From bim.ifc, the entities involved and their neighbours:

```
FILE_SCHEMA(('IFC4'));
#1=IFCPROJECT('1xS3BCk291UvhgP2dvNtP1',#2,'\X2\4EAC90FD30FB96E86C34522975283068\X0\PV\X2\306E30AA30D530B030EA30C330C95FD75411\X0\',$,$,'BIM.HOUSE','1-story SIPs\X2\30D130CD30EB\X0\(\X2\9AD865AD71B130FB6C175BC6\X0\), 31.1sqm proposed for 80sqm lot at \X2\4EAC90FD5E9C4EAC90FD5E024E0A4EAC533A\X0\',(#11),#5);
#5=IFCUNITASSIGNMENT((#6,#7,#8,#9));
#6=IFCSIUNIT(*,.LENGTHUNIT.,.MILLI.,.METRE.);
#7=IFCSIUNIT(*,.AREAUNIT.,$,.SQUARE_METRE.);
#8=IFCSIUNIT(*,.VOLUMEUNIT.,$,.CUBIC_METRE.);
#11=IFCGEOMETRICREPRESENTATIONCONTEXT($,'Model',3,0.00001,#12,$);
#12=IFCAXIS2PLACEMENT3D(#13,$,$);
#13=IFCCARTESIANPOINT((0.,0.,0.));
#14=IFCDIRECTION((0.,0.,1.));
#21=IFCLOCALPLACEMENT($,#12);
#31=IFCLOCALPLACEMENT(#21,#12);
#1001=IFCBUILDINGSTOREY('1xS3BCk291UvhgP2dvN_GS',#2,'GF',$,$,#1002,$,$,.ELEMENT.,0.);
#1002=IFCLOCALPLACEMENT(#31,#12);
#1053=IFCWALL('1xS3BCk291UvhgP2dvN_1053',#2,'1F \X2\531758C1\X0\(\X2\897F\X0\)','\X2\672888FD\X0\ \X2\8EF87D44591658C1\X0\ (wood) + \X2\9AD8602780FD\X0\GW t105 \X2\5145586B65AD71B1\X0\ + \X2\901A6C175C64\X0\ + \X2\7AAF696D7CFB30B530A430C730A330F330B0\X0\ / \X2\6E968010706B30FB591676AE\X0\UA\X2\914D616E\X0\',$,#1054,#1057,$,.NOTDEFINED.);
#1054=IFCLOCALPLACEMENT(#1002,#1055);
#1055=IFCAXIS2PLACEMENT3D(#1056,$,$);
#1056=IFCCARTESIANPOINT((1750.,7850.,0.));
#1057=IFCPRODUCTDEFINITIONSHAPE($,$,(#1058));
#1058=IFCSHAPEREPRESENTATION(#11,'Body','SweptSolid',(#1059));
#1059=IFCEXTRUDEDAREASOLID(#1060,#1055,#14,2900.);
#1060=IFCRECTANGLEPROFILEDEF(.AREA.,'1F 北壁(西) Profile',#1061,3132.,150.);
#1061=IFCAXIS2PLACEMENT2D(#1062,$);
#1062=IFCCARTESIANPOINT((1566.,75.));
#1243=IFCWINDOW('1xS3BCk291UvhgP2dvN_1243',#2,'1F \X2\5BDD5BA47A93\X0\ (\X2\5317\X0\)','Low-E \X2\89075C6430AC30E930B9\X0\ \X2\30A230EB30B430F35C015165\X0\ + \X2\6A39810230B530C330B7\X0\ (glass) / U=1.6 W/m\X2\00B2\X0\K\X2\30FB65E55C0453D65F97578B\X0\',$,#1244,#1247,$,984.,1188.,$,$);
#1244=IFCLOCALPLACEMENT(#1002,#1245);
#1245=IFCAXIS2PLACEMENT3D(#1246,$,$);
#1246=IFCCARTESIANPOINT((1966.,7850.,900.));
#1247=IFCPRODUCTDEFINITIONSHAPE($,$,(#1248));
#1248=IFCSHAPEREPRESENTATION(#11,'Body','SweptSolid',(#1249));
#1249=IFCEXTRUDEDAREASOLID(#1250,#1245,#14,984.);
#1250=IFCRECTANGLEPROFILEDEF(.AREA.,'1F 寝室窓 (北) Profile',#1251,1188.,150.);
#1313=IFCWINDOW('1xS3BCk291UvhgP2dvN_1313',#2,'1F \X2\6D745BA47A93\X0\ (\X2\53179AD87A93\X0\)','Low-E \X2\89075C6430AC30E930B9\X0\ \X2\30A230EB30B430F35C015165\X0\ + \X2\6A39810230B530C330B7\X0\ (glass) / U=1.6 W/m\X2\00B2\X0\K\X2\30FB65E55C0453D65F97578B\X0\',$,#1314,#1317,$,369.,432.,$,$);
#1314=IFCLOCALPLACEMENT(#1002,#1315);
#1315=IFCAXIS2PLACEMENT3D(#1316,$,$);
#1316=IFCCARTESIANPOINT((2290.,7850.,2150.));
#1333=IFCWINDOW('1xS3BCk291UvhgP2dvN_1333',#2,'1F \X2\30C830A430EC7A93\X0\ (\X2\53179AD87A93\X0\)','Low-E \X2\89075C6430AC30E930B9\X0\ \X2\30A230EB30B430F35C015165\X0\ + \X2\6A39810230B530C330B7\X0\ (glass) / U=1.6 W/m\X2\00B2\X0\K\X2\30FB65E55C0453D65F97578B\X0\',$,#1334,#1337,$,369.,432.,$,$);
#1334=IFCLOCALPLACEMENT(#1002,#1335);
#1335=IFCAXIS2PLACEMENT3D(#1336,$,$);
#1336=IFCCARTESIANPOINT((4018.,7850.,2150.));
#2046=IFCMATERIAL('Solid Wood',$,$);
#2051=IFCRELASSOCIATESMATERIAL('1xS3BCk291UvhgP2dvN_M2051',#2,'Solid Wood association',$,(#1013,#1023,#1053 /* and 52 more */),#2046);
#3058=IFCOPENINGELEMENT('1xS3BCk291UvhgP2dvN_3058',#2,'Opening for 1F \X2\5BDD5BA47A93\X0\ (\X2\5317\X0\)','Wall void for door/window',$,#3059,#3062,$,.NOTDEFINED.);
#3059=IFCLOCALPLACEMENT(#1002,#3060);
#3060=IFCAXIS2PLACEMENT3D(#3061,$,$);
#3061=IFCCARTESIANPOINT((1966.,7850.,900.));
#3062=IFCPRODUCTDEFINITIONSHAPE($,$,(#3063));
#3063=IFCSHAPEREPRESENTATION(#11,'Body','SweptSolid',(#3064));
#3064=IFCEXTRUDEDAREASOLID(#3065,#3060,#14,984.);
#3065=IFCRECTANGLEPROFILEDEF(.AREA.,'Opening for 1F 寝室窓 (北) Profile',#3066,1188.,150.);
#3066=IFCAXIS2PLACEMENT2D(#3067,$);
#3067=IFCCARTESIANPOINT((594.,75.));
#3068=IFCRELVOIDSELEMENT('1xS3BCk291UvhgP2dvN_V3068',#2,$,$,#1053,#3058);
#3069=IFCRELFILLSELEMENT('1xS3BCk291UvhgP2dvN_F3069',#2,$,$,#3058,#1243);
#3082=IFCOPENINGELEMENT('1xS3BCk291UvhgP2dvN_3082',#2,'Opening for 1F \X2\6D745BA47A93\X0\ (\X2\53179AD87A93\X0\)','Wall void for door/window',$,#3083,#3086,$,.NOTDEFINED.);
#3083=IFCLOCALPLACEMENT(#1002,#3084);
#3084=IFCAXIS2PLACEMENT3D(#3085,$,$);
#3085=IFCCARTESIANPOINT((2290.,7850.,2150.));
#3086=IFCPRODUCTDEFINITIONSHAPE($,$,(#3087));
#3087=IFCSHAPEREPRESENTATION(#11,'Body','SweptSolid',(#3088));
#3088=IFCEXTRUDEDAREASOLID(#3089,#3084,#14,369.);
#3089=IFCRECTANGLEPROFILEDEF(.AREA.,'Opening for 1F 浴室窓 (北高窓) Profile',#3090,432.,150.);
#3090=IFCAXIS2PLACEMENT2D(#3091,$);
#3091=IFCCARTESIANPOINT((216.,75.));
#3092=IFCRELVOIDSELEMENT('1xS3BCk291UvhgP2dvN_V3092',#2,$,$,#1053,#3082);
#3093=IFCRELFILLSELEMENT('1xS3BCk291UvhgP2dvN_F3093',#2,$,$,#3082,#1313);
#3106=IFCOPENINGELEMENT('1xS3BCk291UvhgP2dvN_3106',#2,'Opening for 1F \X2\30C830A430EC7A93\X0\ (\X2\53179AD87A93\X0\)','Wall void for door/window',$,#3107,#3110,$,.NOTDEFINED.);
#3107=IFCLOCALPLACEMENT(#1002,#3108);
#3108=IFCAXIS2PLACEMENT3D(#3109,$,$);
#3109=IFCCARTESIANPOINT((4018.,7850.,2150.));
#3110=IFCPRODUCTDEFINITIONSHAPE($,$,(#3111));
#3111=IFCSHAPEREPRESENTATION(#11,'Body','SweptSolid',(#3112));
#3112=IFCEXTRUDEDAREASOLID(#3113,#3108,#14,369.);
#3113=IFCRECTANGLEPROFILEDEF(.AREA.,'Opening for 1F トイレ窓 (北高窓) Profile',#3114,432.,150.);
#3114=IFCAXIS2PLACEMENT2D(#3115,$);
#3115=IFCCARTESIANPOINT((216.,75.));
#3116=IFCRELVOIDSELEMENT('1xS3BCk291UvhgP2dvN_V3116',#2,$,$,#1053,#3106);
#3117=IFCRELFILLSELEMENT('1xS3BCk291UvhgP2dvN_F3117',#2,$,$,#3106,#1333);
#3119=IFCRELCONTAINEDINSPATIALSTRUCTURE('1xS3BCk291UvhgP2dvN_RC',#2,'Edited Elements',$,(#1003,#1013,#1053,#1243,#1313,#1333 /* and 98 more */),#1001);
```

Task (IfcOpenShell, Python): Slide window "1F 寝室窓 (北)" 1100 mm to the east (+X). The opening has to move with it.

```python
import ifcopenshell
import ifcopenshell.api.geometry
import ifcopenshell.util.placement
import ifcopenshell.util.unit

model = ifcopenshell.open("bim.ifc")
unit_scale = ifcopenshell.util.unit.calculate_unit_scale(model)

window = model.by_id(1243)
opening = window.FillsVoids[0].RelatingOpeningElement
wall = opening.VoidsElements[0].RelatingBuildingElement

wall_matrix = ifcopenshell.util.placement.get_local_placement(wall.ObjectPlacement)
shift = wall_matrix[:3, 0] * 1.1 / unit_scale
before = ifcopenshell.util.placement.get_local_placement(window.ObjectPlacement)[:3, 3].copy()

# The window is not placed relative to its opening, so move both.
for product in (opening, window):
    matrix = ifcopenshell.util.placement.get_local_placement(product.ObjectPlacement)
    matrix[:3, 3] += shift
    ifcopenshell.api.geometry.edit_object_placement(model, product=product, matrix=matrix, is_si=False)

after = ifcopenshell.util.placement.get_local_placement(window.ObjectPlacement)[:3, 3]
print("window moved by", (after - before).round(3) + 0.0)

model.write("bim_v2.ifc")
```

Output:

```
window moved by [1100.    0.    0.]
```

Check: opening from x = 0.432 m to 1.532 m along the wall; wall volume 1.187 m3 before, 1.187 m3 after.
